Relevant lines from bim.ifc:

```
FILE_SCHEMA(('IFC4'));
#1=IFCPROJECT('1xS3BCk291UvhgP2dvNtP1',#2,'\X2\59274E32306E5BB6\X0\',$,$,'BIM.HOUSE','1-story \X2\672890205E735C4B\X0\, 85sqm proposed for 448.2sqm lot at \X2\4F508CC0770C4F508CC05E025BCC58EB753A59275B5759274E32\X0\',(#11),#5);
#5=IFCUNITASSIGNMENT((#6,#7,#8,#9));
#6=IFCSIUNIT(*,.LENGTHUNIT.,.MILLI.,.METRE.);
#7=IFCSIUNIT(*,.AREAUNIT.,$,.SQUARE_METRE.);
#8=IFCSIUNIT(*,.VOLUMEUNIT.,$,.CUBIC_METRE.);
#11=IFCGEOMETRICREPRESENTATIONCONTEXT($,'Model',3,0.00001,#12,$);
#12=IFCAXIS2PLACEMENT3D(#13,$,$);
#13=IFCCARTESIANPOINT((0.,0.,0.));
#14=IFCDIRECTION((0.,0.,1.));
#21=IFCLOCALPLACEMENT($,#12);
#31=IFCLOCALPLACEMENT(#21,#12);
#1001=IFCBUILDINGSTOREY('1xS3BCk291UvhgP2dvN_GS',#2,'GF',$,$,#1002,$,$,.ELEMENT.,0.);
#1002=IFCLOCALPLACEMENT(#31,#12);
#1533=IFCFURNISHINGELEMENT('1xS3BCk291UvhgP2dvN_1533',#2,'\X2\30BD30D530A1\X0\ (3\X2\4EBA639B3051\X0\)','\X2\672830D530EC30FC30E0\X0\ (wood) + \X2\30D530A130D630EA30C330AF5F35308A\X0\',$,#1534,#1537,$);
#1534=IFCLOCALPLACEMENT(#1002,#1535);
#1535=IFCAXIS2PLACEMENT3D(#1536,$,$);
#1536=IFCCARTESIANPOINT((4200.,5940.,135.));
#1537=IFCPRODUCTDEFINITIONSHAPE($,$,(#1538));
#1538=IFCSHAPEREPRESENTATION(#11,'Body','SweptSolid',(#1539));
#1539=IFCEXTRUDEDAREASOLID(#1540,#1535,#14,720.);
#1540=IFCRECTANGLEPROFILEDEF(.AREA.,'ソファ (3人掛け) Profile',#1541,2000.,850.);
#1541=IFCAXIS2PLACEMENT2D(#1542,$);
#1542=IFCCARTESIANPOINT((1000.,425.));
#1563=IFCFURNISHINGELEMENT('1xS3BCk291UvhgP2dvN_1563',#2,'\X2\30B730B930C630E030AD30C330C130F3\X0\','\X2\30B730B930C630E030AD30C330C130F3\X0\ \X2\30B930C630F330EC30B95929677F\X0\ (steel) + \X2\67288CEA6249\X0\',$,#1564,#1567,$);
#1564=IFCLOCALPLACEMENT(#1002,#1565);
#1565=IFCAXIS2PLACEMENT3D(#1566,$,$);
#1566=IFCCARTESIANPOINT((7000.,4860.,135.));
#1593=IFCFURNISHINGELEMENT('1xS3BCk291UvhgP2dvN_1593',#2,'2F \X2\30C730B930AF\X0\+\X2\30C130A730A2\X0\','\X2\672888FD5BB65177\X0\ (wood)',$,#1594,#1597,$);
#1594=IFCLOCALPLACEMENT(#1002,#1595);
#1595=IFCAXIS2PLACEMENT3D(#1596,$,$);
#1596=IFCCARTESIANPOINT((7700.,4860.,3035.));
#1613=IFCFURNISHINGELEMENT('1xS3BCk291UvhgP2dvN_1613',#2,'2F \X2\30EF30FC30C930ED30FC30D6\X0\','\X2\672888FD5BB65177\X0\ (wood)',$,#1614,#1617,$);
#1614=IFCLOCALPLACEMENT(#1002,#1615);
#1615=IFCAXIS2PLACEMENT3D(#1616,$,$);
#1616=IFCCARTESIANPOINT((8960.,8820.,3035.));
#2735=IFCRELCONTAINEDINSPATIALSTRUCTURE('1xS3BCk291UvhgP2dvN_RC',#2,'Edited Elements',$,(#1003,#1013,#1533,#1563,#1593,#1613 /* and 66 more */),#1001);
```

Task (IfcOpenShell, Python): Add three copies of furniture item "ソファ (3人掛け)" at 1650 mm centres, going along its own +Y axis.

```python
import ifcopenshell
import ifcopenshell.api.geometry
import ifcopenshell.api.root
import ifcopenshell.util.element
import ifcopenshell.util.placement
import ifcopenshell.util.unit

model = ifcopenshell.open("bim.ifc")
unit_scale = ifcopenshell.util.unit.calculate_unit_scale(model)


def reuse_history(source, copy):
    """copy_class also copies each property set's owner history, people and application; keep the originals."""
    for rel in copy.IsDefinedBy:
        if rel.is_a("IfcRelDefinesByProperties") and (history := rel.RelatingPropertyDefinition.OwnerHistory):
            rel.RelatingPropertyDefinition.OwnerHistory = source.OwnerHistory
            ifcopenshell.util.element.remove_deep2(model, history)


source = model.by_guid("1xS3BCk291UvhgP2dvN_1533")
base = ifcopenshell.util.placement.get_local_placement(source.ObjectPlacement)
step = base[:3, 1] * 1.65 / unit_scale

for i in range(1, 4):
    copy = ifcopenshell.api.root.copy_class(model, product=source)
    copy.Representation = ifcopenshell.util.element.copy_deep(
        model, source.Representation, exclude=["IfcGeometricRepresentationContext", "IfcRepresentationMap"]
    )
    reuse_history(source, copy)
    matrix = base.copy()
    matrix[:3, 3] += i * step
    print("added at", matrix[:3, 3].round(3) + 0.0)
    ifcopenshell.api.geometry.edit_object_placement(model, product=copy, matrix=matrix, is_si=False)

model.write("bim-out.ifc")
```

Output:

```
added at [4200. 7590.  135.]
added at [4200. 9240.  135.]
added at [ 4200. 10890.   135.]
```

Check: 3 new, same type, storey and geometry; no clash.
